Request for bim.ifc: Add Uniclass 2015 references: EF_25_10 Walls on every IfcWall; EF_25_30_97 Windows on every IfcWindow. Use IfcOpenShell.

First a look at what the model holds.

```python
import ifcopenshell

model = ifcopenshell.open("bim.ifc")
print(model.schema)
print("classifications:", [c.Name for c in model.by_type("IfcClassification")])
for ifc_class in ("IfcDoor", "IfcRoof", "IfcStair", "IfcWall", "IfcWindow"):
    print(ifc_class, len(model.by_type(ifc_class)))
```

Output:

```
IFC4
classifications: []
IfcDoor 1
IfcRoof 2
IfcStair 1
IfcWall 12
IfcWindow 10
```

```python
import ifcopenshell
import ifcopenshell.api.classification

model = ifcopenshell.open("bim.ifc")

system = ifcopenshell.api.classification.add_classification(model, classification="Uniclass 2015")

codes = {
    "IfcWall": ("EF_25_10", "Walls"),
    "IfcWindow": ("EF_25_30_97", "Windows"),
}
for ifc_class, (code, name) in codes.items():
    products = model.by_type(ifc_class)
    ifcopenshell.api.classification.add_reference(
        model, products=products, classification=system, identification=code, name=name
    )
    print(code, len(products))

model.write("bim_v2.ifc")
```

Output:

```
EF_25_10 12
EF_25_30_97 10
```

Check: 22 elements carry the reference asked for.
